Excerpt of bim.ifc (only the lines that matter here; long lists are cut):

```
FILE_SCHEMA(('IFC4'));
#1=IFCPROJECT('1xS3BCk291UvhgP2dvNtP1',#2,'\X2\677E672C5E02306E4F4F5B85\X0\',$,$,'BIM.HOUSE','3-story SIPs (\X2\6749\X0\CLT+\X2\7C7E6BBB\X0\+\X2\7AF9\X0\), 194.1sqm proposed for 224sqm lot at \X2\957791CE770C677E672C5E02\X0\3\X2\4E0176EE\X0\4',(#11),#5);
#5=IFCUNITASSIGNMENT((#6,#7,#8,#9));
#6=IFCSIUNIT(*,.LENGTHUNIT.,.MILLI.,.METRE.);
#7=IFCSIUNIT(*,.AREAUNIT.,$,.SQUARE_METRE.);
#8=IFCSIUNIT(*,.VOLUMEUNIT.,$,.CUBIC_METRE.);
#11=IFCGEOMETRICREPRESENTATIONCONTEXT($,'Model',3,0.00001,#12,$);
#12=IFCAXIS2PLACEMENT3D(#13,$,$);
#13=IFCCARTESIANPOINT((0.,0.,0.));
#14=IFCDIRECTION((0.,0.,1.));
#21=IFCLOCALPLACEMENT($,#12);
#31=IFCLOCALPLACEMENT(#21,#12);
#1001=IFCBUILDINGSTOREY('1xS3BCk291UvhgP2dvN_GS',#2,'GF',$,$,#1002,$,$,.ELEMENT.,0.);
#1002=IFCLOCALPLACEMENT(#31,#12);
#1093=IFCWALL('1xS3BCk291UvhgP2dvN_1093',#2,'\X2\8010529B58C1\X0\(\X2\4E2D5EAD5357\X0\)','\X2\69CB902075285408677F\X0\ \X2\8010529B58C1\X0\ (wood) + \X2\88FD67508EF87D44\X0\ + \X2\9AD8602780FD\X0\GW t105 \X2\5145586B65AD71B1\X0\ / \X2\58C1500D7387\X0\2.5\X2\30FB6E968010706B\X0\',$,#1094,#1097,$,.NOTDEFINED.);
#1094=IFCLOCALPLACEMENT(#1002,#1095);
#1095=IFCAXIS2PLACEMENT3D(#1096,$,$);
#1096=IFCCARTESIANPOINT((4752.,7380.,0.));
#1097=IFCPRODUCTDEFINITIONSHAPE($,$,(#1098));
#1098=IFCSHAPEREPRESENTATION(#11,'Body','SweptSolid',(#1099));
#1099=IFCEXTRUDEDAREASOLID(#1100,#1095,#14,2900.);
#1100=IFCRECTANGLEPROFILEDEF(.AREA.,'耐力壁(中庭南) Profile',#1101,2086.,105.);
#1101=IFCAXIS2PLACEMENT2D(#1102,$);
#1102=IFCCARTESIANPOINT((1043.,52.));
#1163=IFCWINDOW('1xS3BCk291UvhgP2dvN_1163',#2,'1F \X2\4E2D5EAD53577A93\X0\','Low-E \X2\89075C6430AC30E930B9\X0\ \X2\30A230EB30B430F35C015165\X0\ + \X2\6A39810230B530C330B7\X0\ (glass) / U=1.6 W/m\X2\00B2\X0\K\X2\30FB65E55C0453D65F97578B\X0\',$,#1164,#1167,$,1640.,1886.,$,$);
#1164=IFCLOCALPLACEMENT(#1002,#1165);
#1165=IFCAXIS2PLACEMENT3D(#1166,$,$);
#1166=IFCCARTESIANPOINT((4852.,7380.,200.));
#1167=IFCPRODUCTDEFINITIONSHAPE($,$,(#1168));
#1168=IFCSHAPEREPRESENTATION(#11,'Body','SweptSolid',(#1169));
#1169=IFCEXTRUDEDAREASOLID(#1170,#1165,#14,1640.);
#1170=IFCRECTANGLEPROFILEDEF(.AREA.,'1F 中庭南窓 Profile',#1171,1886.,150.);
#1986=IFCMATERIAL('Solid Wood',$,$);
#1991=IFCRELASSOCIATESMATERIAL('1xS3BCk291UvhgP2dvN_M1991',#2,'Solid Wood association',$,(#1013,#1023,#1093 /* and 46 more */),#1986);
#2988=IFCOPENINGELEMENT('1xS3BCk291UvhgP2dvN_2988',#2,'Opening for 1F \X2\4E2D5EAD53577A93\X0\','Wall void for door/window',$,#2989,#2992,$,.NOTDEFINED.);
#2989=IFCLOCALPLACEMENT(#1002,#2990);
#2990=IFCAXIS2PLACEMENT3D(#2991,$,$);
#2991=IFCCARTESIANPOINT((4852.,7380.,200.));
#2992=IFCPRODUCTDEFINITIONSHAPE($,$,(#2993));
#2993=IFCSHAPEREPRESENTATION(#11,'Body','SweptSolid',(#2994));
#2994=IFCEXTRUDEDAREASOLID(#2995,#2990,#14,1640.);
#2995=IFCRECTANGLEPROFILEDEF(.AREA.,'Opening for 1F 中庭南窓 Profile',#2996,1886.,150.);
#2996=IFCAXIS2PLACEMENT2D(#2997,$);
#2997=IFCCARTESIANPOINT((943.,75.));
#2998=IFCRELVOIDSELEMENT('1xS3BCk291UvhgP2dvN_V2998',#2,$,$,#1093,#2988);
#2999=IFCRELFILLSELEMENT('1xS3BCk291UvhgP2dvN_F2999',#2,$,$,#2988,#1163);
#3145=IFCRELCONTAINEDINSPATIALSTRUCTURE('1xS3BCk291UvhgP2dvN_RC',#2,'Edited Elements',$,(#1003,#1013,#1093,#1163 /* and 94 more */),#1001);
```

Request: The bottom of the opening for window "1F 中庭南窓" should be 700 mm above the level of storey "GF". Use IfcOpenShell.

```python
import numpy as np
import ifcopenshell
import ifcopenshell.api.geometry
import ifcopenshell.geom
import ifcopenshell.util.element
import ifcopenshell.util.placement
import ifcopenshell.util.shape
import ifcopenshell.util.unit

model = ifcopenshell.open("bim.ifc")
unit_scale = ifcopenshell.util.unit.calculate_unit_scale(model)

window = model.by_guid("1xS3BCk291UvhgP2dvN_1163")
opening = window.FillsVoids[0].RelatingOpeningElement
storey = ifcopenshell.util.element.get_container(window, ifc_class="IfcBuildingStorey")
level = ifcopenshell.util.placement.get_local_placement(storey.ObjectPlacement)[2, 3]

# The opening's origin need not be at the sill, so measure its lowest point.
shape = ifcopenshell.geom.create_shape(ifcopenshell.geom.settings(), opening)
bottom = ifcopenshell.util.shape.get_shape_bottom_elevation(shape, shape.geometry) / unit_scale
dz = level + 0.7 / unit_scale - bottom

shift = np.array([0.0, 0.0, dz])
# The window is not placed relative to its opening, so move both.
for product in (opening, window):
    matrix = ifcopenshell.util.placement.get_local_placement(product.ObjectPlacement)
    matrix[:3, 3] += shift
    ifcopenshell.api.geometry.edit_object_placement(model, product=product, matrix=matrix, is_si=False)

print(f"moved by {dz * unit_scale:+.3f} m")

model.write("bim_edited.ifc")
```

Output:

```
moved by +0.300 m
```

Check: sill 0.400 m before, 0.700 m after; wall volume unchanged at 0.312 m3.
